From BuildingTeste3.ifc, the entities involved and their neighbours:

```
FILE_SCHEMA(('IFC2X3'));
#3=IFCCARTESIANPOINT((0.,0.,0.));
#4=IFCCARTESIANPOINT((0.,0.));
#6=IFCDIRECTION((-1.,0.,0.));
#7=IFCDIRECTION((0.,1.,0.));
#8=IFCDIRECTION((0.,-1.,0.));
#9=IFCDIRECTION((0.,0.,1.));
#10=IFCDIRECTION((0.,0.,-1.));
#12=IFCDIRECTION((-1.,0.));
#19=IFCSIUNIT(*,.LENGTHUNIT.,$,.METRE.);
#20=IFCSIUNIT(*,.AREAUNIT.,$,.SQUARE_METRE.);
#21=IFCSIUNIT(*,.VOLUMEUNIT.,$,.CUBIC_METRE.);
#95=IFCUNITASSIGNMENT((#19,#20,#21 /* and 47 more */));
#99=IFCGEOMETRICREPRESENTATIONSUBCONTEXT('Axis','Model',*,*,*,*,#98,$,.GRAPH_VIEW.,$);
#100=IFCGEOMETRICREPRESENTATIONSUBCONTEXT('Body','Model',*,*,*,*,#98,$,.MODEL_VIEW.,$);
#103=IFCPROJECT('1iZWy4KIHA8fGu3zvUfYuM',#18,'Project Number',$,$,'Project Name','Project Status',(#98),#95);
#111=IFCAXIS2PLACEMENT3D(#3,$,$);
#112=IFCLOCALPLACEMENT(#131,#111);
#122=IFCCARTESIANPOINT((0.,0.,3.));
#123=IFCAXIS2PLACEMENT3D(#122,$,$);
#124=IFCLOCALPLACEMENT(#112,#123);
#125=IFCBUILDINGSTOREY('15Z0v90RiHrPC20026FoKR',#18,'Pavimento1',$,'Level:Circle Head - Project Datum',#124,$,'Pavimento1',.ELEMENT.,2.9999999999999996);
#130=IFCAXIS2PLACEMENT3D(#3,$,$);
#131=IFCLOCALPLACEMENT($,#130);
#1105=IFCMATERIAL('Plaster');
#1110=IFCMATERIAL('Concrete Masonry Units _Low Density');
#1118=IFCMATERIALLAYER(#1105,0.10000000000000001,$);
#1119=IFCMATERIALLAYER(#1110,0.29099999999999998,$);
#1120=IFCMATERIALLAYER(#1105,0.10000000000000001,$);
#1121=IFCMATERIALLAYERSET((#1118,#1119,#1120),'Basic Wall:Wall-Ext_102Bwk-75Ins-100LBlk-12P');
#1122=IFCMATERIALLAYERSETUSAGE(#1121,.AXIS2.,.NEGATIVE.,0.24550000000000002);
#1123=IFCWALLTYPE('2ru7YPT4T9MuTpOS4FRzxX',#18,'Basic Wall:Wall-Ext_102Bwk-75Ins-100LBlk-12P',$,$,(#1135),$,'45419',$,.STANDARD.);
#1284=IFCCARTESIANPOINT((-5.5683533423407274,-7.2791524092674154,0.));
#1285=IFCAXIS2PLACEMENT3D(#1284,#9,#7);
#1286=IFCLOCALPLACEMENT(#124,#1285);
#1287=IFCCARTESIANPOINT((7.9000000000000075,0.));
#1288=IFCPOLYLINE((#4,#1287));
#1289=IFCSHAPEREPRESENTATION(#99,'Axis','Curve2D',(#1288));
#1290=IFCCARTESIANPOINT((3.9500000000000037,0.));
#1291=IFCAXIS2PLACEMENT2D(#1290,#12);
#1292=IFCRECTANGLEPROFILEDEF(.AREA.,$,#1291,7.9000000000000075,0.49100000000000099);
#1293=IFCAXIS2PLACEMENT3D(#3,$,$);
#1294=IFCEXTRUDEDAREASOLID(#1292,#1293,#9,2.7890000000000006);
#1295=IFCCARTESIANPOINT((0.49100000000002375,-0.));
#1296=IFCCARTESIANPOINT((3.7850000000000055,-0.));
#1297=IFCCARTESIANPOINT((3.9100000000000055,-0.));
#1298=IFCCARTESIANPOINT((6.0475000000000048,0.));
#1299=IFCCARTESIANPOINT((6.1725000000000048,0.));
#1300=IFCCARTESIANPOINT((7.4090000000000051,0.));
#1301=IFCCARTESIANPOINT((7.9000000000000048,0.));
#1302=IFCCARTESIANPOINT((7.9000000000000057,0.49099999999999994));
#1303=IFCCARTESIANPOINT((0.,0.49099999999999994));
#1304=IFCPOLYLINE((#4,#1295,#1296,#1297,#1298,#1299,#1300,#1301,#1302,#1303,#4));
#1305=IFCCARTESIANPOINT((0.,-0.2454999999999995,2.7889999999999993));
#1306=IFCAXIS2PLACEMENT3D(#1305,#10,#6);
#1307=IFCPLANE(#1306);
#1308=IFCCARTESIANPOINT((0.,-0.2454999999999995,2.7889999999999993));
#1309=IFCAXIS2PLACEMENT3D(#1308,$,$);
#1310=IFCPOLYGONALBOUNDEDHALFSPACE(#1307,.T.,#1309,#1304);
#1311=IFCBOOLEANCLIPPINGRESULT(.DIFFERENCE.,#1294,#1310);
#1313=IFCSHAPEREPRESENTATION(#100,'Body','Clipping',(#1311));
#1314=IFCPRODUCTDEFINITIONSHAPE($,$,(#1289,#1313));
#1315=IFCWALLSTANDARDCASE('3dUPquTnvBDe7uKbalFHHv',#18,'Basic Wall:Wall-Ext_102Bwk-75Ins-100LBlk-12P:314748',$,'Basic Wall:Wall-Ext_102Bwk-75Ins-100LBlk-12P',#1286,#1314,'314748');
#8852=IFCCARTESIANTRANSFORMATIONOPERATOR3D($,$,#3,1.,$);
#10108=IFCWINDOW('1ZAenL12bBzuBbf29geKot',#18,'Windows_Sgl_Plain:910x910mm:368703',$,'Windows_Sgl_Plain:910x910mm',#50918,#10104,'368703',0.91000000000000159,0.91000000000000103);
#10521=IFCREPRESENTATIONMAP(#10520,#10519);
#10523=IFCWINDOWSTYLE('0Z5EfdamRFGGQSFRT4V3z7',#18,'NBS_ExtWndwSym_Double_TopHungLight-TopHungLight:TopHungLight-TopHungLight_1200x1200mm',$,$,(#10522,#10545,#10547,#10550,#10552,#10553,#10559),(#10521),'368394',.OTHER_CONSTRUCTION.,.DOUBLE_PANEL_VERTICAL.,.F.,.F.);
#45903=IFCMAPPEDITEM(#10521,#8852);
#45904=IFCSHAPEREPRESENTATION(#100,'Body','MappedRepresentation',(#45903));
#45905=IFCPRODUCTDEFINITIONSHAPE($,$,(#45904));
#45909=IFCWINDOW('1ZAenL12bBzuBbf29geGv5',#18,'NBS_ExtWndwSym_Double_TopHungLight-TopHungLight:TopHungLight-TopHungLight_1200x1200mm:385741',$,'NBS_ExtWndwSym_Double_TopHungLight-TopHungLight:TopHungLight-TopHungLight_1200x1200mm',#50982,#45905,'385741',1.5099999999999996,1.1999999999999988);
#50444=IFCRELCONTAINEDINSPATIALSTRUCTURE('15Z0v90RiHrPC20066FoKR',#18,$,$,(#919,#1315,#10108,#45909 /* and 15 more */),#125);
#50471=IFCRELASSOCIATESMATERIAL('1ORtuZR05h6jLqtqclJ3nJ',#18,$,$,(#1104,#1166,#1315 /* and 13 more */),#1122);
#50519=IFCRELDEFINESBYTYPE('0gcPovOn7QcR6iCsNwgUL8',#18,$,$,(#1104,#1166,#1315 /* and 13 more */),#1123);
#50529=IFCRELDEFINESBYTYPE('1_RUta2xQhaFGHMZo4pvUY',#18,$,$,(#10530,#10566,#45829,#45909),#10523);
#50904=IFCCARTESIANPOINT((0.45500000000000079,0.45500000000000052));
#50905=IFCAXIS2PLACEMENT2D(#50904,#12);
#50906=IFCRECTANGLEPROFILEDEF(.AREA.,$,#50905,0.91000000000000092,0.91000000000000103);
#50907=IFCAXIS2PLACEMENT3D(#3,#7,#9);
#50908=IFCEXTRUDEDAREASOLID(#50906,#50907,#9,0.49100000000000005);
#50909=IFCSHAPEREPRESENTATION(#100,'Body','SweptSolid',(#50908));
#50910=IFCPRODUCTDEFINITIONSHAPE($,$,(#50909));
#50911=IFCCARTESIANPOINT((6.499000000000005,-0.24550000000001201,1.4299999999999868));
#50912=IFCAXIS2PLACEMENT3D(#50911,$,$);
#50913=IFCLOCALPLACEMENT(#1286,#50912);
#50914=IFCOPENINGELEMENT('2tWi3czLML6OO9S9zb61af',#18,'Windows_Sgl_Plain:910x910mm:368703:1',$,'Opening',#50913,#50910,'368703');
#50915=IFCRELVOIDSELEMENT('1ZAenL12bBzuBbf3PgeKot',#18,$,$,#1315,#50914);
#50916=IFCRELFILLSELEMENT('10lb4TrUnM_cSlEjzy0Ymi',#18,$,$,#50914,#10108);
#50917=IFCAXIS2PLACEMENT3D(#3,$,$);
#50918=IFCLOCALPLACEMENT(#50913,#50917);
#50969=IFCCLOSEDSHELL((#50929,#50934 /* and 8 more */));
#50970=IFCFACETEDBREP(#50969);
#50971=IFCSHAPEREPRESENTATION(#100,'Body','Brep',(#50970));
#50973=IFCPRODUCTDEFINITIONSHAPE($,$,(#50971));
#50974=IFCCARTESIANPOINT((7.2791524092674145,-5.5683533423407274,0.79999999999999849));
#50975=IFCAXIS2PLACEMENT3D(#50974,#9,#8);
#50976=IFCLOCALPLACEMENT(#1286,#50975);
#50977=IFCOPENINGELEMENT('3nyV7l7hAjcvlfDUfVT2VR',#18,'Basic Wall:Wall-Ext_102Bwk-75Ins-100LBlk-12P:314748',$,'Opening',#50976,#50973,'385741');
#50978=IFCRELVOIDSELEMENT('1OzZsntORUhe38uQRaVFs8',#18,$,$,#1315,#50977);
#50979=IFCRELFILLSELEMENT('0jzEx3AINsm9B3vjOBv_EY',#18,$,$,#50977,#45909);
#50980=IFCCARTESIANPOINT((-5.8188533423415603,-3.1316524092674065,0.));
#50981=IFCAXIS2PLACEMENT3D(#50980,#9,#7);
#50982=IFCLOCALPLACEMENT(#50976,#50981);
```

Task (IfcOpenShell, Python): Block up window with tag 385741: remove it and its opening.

```python
import ifcopenshell
import ifcopenshell.api.feature
import ifcopenshell.api.root
import ifcopenshell.geom
import ifcopenshell.util.shape

model = ifcopenshell.open("BuildingTeste3.ifc")
settings = ifcopenshell.geom.settings()


def volume(element):
    """Net volume in cubic metres, openings subtracted."""
    shape = ifcopenshell.geom.create_shape(settings, element)
    return ifcopenshell.util.shape.get_volume(shape.geometry)


window = model.by_guid("1ZAenL12bBzuBbf29geGv5")
opening = window.FillsVoids[0].RelatingOpeningElement
wall = opening.VoidsElements[0].RelatingBuildingElement
before = volume(wall)

ifcopenshell.api.root.remove_product(model, product=window)
ifcopenshell.api.feature.remove_feature(model, feature=opening)

after = volume(wall)

print(f"wall volume {before:.3f} -> {after:.3f} m3")

model.write("BuildingTeste3_updated.ifc")
```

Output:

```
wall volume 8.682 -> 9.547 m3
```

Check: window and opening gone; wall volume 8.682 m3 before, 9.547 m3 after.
